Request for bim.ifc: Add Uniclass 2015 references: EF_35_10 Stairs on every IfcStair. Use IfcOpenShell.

First a look at what the model holds.

```python
import ifcopenshell

model = ifcopenshell.open("bim.ifc")
print(model.schema)
print("classifications:", [c.Name for c in model.by_type("IfcClassification")])
for ifc_class in ("IfcDoor", "IfcRoof", "IfcStair", "IfcWall", "IfcWindow"):
    print(ifc_class, len(model.by_type(ifc_class)))
```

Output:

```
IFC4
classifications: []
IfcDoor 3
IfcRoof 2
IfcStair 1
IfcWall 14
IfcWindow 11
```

```python
import ifcopenshell
import ifcopenshell.api.classification

model = ifcopenshell.open("bim.ifc")

system = ifcopenshell.api.classification.add_classification(model, classification="Uniclass 2015")

codes = {
    "IfcStair": ("EF_35_10", "Stairs"),
}
for ifc_class, (code, name) in codes.items():
    products = model.by_type(ifc_class)
    ifcopenshell.api.classification.add_reference(
        model, products=products, classification=system, identification=code, name=name
    )
    print(code, len(products))

model.write("bim_updated.ifc")
```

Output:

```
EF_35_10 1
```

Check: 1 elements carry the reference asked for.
